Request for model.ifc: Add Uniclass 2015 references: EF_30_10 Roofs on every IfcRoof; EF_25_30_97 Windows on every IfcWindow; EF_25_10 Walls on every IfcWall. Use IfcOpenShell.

First a look at what the model holds.

```python
import ifcopenshell

model = ifcopenshell.open("model.ifc")
print(model.schema)
print("classifications:", [c.Name for c in model.by_type("IfcClassification")])
for ifc_class in ("IfcDoor", "IfcRoof", "IfcStair", "IfcWall", "IfcWindow"):
    print(ifc_class, len(model.by_type(ifc_class)))
```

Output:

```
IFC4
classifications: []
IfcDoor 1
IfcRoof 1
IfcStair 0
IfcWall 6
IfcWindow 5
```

```python
import ifcopenshell
import ifcopenshell.api.classification

model = ifcopenshell.open("model.ifc")

system = ifcopenshell.api.classification.add_classification(model, classification="Uniclass 2015")

codes = {
    "IfcRoof": ("EF_30_10", "Roofs"),
    "IfcWindow": ("EF_25_30_97", "Windows"),
    "IfcWall": ("EF_25_10", "Walls"),
}
for ifc_class, (code, name) in codes.items():
    products = model.by_type(ifc_class)
    ifcopenshell.api.classification.add_reference(
        model, products=products, classification=system, identification=code, name=name
    )
    print(code, len(products))

model.write("model_updated.ifc")
```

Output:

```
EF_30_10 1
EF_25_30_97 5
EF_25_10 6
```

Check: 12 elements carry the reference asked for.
